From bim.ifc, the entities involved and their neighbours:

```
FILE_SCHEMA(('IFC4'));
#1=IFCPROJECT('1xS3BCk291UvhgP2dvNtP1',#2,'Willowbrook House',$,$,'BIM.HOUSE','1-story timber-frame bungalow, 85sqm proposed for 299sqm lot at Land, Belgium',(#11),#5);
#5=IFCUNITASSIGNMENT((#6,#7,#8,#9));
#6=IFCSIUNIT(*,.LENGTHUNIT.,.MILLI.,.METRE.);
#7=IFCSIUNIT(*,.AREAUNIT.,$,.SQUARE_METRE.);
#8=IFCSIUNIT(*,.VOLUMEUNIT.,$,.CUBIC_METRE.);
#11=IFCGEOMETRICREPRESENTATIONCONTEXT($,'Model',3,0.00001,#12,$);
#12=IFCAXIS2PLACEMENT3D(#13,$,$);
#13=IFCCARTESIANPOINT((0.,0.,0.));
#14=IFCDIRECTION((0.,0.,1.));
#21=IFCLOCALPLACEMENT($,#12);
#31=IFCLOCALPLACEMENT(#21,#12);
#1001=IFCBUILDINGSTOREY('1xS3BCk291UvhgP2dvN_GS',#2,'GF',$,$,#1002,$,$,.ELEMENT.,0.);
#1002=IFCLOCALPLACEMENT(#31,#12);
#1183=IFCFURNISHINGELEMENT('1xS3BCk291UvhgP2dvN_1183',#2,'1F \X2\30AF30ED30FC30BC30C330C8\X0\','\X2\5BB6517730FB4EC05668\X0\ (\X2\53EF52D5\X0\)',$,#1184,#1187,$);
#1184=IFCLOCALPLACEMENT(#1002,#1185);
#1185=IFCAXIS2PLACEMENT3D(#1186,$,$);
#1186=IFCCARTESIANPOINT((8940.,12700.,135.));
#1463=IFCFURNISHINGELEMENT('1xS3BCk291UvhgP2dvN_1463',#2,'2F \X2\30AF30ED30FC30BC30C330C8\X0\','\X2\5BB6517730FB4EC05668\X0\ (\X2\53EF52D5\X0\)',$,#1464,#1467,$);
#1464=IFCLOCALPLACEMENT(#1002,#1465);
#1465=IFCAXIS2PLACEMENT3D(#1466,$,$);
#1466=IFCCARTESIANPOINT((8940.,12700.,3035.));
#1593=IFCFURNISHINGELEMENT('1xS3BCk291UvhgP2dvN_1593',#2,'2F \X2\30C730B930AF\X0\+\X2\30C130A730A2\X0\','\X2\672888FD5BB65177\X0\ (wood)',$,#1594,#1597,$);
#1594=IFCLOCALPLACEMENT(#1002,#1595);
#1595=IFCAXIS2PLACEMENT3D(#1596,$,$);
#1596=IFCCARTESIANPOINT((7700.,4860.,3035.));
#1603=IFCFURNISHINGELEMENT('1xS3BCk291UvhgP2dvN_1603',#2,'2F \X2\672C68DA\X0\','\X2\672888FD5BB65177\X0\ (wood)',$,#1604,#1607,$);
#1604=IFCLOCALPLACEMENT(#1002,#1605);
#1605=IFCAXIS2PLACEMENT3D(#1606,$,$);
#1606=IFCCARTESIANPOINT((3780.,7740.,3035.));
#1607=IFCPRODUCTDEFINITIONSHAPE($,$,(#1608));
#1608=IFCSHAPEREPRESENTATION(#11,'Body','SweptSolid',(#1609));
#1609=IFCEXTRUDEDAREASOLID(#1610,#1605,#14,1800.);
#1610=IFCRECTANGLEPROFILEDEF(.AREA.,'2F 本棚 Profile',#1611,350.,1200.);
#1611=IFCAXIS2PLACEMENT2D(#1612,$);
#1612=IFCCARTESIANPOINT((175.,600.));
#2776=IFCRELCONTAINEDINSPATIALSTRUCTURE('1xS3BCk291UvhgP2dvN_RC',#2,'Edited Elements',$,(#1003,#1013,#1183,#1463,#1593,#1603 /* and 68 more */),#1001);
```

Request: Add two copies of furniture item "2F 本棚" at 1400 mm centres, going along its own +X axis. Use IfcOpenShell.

```python
import ifcopenshell
import ifcopenshell.api.geometry
import ifcopenshell.api.root
import ifcopenshell.util.element
import ifcopenshell.util.placement
import ifcopenshell.util.unit

model = ifcopenshell.open("bim.ifc")
unit_scale = ifcopenshell.util.unit.calculate_unit_scale(model)


def reuse_history(source, copy):
    """copy_class also copies each property set's owner history, people and application; keep the originals."""
    for rel in copy.IsDefinedBy:
        if rel.is_a("IfcRelDefinesByProperties") and (history := rel.RelatingPropertyDefinition.OwnerHistory):
            rel.RelatingPropertyDefinition.OwnerHistory = source.OwnerHistory
            ifcopenshell.util.element.remove_deep2(model, history)


source = model.by_guid("1xS3BCk291UvhgP2dvN_1603")
base = ifcopenshell.util.placement.get_local_placement(source.ObjectPlacement)
step = base[:3, 0] * 1.4 / unit_scale

for i in range(1, 3):
    copy = ifcopenshell.api.root.copy_class(model, product=source)
    copy.Representation = ifcopenshell.util.element.copy_deep(
        model, source.Representation, exclude=["IfcGeometricRepresentationContext", "IfcRepresentationMap"]
    )
    reuse_history(source, copy)
    matrix = base.copy()
    matrix[:3, 3] += i * step
    print("added at", matrix[:3, 3].round(3) + 0.0)
    ifcopenshell.api.geometry.edit_object_placement(model, product=copy, matrix=matrix, is_si=False)

model.write("bim_edited.ifc")
```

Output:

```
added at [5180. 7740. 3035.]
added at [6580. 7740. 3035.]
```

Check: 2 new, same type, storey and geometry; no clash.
